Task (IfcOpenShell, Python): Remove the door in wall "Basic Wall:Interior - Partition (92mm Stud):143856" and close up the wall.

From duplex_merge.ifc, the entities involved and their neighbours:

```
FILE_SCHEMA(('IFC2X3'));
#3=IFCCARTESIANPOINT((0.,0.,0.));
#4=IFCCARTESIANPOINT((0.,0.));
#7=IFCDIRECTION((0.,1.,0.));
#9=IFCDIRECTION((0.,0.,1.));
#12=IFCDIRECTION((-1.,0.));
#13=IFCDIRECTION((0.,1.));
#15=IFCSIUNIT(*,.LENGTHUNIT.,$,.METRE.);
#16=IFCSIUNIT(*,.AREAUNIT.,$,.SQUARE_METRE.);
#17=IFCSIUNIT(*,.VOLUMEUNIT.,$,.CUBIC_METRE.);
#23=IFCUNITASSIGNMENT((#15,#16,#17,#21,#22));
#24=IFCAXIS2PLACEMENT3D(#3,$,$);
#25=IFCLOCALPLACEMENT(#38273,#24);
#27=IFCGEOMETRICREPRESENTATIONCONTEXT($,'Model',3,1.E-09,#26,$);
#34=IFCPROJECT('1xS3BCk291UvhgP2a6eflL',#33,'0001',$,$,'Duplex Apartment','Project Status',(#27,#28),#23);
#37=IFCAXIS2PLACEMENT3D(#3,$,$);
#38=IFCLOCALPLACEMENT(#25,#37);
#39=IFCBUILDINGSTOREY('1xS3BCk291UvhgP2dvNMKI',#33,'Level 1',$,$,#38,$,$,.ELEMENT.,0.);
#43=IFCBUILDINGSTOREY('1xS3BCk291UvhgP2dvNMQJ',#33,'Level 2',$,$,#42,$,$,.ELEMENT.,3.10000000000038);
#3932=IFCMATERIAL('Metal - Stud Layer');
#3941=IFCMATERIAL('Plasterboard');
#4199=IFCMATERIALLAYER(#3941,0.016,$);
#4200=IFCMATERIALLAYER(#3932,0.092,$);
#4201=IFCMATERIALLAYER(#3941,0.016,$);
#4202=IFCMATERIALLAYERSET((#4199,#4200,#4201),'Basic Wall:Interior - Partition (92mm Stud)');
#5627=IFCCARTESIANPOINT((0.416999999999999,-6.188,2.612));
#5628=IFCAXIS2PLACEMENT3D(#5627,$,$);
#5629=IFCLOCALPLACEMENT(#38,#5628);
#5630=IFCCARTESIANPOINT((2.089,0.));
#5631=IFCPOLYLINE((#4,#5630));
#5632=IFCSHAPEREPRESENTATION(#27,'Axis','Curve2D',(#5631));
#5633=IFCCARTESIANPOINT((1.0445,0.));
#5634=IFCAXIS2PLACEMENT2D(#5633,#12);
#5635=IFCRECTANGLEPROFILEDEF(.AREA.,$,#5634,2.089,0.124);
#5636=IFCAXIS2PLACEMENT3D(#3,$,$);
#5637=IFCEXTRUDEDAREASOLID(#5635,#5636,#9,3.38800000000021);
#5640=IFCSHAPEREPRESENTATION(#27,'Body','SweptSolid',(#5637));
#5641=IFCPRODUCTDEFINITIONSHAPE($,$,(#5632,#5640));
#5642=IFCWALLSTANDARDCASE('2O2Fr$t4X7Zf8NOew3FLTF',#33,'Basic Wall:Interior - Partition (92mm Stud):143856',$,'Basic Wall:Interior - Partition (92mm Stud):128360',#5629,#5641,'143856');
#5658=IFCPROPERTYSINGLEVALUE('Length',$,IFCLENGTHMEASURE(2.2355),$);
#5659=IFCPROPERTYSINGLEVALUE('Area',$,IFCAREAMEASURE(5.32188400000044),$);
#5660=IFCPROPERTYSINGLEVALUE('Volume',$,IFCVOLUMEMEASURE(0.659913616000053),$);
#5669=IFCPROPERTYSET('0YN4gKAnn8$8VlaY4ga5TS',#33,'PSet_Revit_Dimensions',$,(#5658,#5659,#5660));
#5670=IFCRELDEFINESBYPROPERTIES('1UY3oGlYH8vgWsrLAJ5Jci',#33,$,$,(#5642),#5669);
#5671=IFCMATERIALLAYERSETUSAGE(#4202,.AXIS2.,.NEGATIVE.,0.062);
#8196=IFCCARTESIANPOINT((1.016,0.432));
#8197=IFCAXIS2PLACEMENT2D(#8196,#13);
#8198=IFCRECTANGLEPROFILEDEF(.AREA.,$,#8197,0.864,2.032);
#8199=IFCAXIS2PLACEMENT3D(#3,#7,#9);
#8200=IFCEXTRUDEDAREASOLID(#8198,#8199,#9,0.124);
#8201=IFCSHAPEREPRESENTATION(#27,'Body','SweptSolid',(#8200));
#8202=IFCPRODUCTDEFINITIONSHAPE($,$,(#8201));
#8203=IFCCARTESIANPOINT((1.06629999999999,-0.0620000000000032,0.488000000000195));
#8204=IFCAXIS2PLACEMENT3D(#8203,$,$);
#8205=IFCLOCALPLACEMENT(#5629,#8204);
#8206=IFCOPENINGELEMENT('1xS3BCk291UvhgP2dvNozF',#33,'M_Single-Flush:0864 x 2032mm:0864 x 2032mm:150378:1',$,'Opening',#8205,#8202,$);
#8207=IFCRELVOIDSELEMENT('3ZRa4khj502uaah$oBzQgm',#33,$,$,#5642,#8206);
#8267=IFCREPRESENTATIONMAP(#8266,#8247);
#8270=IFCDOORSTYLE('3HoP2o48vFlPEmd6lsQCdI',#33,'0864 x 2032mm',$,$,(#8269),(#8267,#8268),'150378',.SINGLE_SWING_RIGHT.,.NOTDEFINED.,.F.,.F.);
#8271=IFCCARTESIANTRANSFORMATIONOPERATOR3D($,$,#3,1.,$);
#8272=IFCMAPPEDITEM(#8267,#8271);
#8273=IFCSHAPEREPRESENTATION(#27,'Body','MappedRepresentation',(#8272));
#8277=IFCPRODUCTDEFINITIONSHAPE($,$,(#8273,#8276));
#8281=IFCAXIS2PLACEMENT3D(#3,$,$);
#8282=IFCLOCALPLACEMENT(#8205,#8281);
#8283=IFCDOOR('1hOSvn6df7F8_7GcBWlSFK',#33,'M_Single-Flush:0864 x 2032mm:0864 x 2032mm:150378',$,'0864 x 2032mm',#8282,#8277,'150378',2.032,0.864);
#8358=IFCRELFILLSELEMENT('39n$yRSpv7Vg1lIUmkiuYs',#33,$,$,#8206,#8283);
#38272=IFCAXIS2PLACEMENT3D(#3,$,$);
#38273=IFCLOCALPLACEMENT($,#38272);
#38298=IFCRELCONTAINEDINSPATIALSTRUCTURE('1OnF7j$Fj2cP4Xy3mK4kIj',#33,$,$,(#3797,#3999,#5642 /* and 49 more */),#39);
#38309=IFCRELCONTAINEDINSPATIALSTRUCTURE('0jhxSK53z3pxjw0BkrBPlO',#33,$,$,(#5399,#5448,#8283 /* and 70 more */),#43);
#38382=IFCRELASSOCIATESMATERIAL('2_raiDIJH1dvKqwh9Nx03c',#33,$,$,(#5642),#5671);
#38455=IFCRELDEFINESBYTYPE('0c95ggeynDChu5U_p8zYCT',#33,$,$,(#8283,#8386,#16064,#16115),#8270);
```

```python
import ifcopenshell
import ifcopenshell.api.feature
import ifcopenshell.api.pset
import ifcopenshell.api.root
import ifcopenshell.geom
import ifcopenshell.util.element
import ifcopenshell.util.shape
import ifcopenshell.util.unit

model = ifcopenshell.open("duplex_merge.ifc")
area_scale = ifcopenshell.util.unit.calculate_unit_scale(model, "AREAUNIT")
volume_scale = ifcopenshell.util.unit.calculate_unit_scale(model, "VOLUMEUNIT")
settings = ifcopenshell.geom.settings()


def volume(element):
    """Net volume in cubic metres, openings subtracted."""
    shape = ifcopenshell.geom.create_shape(settings, element)
    return ifcopenshell.util.shape.get_volume(shape.geometry)


door = model.by_guid("1hOSvn6df7F8_7GcBWlSFK")
opening = door.FillsVoids[0].RelatingOpeningElement
wall = opening.VoidsElements[0].RelatingBuildingElement
before = volume(wall)

ifcopenshell.api.root.remove_product(model, product=door)
ifcopenshell.api.feature.remove_feature(model, feature=opening)

after = volume(wall)
thickness = 0.124  # wall thickness in metres

# Update the wall's stored quantities.
pset = model.by_id(ifcopenshell.util.element.get_pset(wall, "PSet_Revit_Dimensions", should_inherit=False)["id"])
ifcopenshell.api.pset.edit_pset(model, pset=pset, properties={
    "Area": model.create_entity("IfcAreaMeasure", after / thickness / area_scale),
    "Volume": model.create_entity("IfcVolumeMeasure", after / volume_scale),
})

print(f"wall volume {before:.3f} -> {after:.3f} m3")

model.write("duplex_merge-out.ifc")
```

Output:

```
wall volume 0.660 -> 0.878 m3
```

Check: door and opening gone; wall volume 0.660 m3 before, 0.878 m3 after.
